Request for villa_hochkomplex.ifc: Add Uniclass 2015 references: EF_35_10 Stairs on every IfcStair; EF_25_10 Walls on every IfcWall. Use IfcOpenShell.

First a look at what the model holds.

```python
import ifcopenshell

model = ifcopenshell.open("villa_hochkomplex.ifc")
print(model.schema)
print("classifications:", [c.Name for c in model.by_type("IfcClassification")])
for ifc_class in ("IfcDoor", "IfcRoof", "IfcStair", "IfcWall", "IfcWindow"):
    print(ifc_class, len(model.by_type(ifc_class)))
```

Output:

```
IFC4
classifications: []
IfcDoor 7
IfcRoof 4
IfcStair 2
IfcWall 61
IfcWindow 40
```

```python
import ifcopenshell
import ifcopenshell.api.classification

model = ifcopenshell.open("villa_hochkomplex.ifc")

system = ifcopenshell.api.classification.add_classification(model, classification="Uniclass 2015")

codes = {
    "IfcStair": ("EF_35_10", "Stairs"),
    "IfcWall": ("EF_25_10", "Walls"),
}
for ifc_class, (code, name) in codes.items():
    products = model.by_type(ifc_class)
    ifcopenshell.api.classification.add_reference(
        model, products=products, classification=system, identification=code, name=name
    )
    print(code, len(products))

model.write("villa_hochkomplex-out.ifc")
```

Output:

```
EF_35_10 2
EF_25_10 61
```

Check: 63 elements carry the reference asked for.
